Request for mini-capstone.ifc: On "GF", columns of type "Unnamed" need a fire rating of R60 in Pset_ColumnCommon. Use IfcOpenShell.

First a look at what the model holds.

```python
import ifcopenshell
import ifcopenshell.util.element

model = ifcopenshell.open("mini-capstone.ifc")
print(model.schema)
storey = next(s for s in model.by_type("IfcBuildingStorey") if s.Name == "GF")
columns = [e for e in ifcopenshell.util.element.get_decomposition(storey) if e.is_a("IfcColumn")]
seen = {}
for e in columns:
    element_type = ifcopenshell.util.element.get_type(e)
    key = (element_type.Name if element_type != e and element_type else None, ifcopenshell.util.element.get_pset(e, "Pset_ColumnCommon", "FireRating"))
    seen[key] = seen.get(key, 0) + 1
for (name, value), count in sorted(seen.items(), key=str):
    print(count, "x", name, "|", value)
```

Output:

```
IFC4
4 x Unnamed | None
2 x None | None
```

```python
import ifcopenshell
import ifcopenshell.api.pset
import ifcopenshell.util.element

model = ifcopenshell.open("mini-capstone.ifc")

storey = next(s for s in model.by_type("IfcBuildingStorey") if s.Name == "GF")
columns = [e for e in ifcopenshell.util.element.get_decomposition(storey) if e.is_a("IfcColumn")]

count = 0
for e in columns:
    element_type = ifcopenshell.util.element.get_type(e)
    if element_type in (None, e) or element_type.Name != "Unnamed":
        continue
    # add_pset returns the element's existing set when there is one.
    pset = ifcopenshell.api.pset.add_pset(model, product=e, name="Pset_ColumnCommon")
    ifcopenshell.api.pset.edit_pset(model, pset=pset, properties={"FireRating": "R60"})
    count += 1

print(count, "columns updated")

model.write("mini-capstone_v2.ifc")
```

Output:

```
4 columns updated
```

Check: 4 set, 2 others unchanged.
